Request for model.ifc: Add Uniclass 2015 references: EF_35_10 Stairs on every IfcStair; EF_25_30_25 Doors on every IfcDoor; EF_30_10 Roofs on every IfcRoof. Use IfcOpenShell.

First a look at what the model holds.

```python
import ifcopenshell

model = ifcopenshell.open("model.ifc")
print(model.schema)
print("classifications:", [c.Name for c in model.by_type("IfcClassification")])
for ifc_class in ("IfcDoor", "IfcRoof", "IfcStair", "IfcWall", "IfcWindow"):
    print(ifc_class, len(model.by_type(ifc_class)))
```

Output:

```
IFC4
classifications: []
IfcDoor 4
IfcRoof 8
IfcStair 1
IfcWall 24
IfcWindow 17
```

```python
import ifcopenshell
import ifcopenshell.api.classification

model = ifcopenshell.open("model.ifc")

system = ifcopenshell.api.classification.add_classification(model, classification="Uniclass 2015")

codes = {
    "IfcStair": ("EF_35_10", "Stairs"),
    "IfcDoor": ("EF_25_30_25", "Doors"),
    "IfcRoof": ("EF_30_10", "Roofs"),
}
for ifc_class, (code, name) in codes.items():
    products = model.by_type(ifc_class)
    ifcopenshell.api.classification.add_reference(
        model, products=products, classification=system, identification=code, name=name
    )
    print(code, len(products))

model.write("model_edited.ifc")
```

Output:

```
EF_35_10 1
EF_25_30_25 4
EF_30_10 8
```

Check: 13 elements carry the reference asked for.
